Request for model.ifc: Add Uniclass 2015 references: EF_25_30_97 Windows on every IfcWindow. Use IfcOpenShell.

First a look at what the model holds.

```python
import ifcopenshell

model = ifcopenshell.open("model.ifc")
print(model.schema)
print("classifications:", [c.Name for c in model.by_type("IfcClassification")])
for ifc_class in ("IfcDoor", "IfcRoof", "IfcStair", "IfcWall", "IfcWindow"):
    print(ifc_class, len(model.by_type(ifc_class)))
```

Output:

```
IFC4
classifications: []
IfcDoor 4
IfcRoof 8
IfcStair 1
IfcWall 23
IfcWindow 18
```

```python
import ifcopenshell
import ifcopenshell.api.classification

model = ifcopenshell.open("model.ifc")

system = ifcopenshell.api.classification.add_classification(model, classification="Uniclass 2015")

codes = {
    "IfcWindow": ("EF_25_30_97", "Windows"),
}
for ifc_class, (code, name) in codes.items():
    products = model.by_type(ifc_class)
    ifcopenshell.api.classification.add_reference(
        model, products=products, classification=system, identification=code, name=name
    )
    print(code, len(products))

model.write("model_edited.ifc")
```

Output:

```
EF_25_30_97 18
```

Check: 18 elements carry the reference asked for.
